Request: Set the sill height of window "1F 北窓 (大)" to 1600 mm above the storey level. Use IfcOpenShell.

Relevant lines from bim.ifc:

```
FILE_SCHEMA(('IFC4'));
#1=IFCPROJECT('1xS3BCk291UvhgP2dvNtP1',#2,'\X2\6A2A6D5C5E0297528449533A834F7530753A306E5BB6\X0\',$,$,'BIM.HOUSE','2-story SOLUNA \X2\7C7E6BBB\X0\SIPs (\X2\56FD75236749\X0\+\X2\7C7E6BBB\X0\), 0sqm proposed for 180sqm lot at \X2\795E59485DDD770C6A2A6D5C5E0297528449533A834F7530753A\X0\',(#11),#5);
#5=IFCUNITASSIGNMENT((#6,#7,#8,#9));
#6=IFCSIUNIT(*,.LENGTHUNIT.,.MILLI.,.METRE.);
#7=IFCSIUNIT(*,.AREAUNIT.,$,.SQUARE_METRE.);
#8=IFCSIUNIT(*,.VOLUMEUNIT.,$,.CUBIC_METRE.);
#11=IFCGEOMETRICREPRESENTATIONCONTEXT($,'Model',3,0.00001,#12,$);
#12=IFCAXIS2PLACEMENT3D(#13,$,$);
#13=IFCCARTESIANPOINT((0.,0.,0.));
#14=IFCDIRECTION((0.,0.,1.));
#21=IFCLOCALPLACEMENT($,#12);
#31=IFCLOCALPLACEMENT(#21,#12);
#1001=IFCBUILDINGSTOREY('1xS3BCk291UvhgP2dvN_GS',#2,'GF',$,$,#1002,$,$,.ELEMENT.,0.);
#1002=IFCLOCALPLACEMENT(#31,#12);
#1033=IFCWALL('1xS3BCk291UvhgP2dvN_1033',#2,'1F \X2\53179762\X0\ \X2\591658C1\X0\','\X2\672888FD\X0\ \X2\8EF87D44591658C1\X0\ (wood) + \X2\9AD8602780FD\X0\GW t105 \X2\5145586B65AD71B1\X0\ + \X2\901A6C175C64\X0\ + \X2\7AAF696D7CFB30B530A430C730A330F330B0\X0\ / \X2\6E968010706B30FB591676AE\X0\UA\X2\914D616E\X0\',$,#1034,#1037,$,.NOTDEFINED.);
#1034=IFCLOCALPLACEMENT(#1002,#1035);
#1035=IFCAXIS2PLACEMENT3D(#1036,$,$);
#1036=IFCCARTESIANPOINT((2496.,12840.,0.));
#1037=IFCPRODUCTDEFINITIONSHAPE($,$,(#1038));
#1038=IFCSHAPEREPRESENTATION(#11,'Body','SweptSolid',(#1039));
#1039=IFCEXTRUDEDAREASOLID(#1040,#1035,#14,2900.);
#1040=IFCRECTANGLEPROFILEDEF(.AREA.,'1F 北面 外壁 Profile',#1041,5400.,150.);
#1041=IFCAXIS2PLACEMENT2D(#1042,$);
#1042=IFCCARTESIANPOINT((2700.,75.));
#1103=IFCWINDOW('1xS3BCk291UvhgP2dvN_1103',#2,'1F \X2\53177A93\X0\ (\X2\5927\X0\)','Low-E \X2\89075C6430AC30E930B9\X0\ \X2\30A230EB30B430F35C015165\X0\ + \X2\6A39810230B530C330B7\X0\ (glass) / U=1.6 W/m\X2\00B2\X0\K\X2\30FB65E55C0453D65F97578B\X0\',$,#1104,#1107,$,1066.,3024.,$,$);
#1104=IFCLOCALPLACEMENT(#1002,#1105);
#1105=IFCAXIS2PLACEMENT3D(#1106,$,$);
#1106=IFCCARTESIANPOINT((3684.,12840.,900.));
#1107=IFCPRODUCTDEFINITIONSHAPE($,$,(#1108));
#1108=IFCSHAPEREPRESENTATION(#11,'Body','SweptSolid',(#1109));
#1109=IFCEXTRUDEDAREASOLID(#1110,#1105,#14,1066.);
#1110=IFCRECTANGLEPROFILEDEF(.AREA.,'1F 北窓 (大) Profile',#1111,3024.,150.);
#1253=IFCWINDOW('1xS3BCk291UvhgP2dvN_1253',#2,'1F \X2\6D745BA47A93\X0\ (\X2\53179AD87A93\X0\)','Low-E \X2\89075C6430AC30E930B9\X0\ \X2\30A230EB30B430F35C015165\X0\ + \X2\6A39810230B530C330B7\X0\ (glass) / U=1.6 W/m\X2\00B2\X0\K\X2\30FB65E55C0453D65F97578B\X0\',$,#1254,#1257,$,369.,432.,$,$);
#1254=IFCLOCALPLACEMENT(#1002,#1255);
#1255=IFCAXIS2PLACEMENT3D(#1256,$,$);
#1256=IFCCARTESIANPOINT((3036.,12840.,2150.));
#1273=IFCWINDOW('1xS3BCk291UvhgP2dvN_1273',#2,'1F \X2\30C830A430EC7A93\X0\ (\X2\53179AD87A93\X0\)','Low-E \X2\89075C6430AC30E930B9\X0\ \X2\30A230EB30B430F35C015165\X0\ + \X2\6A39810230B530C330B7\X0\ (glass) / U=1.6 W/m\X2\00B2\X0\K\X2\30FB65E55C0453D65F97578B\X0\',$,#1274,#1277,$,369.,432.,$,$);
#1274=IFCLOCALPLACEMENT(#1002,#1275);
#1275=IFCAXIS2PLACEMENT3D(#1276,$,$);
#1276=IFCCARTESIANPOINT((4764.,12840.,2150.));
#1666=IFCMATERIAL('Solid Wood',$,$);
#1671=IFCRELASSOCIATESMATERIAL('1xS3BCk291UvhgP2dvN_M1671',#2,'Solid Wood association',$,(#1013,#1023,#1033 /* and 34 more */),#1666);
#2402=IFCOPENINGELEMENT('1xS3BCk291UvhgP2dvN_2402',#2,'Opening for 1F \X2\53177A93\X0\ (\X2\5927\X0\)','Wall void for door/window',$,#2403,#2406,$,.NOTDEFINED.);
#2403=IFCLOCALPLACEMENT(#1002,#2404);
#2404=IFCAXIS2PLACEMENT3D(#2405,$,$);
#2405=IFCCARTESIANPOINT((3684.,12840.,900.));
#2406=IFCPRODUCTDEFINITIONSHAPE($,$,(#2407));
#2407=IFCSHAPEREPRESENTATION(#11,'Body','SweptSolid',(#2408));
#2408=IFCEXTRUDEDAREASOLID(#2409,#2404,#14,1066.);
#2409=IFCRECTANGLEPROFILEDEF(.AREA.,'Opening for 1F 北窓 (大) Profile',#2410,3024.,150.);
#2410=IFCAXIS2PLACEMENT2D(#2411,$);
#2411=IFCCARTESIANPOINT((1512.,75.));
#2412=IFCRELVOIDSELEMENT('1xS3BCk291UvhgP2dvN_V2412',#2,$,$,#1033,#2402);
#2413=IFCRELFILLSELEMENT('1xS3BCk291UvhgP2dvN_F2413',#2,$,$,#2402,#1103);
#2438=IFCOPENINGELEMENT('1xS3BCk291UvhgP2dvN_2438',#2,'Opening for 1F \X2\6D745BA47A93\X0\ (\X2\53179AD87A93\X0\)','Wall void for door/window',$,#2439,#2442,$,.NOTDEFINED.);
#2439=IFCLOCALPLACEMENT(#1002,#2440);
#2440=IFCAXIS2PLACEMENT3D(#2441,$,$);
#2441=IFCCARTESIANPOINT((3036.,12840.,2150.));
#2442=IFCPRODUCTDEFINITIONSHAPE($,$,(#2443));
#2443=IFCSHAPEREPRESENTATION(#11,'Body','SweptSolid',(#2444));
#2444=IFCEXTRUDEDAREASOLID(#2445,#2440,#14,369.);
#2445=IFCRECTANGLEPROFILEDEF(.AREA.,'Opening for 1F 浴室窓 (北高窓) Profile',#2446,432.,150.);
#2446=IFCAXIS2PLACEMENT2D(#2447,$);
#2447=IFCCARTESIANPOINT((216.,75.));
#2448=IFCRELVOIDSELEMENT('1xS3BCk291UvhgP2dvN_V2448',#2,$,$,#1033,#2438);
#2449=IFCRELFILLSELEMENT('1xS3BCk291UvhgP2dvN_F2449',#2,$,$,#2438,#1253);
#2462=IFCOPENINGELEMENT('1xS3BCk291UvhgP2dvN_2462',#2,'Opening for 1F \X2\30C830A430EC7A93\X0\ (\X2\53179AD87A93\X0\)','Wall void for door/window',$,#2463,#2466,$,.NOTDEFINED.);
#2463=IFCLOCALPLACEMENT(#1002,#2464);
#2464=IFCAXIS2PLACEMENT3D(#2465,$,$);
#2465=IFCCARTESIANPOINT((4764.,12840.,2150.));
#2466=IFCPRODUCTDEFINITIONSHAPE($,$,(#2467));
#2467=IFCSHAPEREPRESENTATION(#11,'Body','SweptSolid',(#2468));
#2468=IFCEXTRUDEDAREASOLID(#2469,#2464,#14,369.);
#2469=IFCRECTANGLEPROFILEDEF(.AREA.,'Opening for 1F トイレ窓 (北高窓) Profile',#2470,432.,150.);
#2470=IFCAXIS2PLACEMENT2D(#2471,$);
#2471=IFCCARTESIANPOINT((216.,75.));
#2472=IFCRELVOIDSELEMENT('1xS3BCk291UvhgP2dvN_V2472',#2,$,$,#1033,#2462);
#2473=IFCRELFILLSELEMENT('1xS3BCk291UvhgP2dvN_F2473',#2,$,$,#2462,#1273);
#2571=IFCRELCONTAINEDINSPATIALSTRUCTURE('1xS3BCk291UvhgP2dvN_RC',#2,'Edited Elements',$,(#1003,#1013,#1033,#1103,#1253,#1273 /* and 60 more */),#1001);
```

```python
import numpy as np
import ifcopenshell
import ifcopenshell.api.geometry
import ifcopenshell.geom
import ifcopenshell.util.element
import ifcopenshell.util.placement
import ifcopenshell.util.shape
import ifcopenshell.util.unit

model = ifcopenshell.open("bim.ifc")
unit_scale = ifcopenshell.util.unit.calculate_unit_scale(model)

window = model.by_guid("1xS3BCk291UvhgP2dvN_1103")
opening = window.FillsVoids[0].RelatingOpeningElement
storey = ifcopenshell.util.element.get_container(window, ifc_class="IfcBuildingStorey")
level = ifcopenshell.util.placement.get_local_placement(storey.ObjectPlacement)[2, 3]

# The opening's origin need not be at the sill, so measure its lowest point.
shape = ifcopenshell.geom.create_shape(ifcopenshell.geom.settings(), opening)
bottom = ifcopenshell.util.shape.get_shape_bottom_elevation(shape, shape.geometry) / unit_scale
dz = level + 1.6 / unit_scale - bottom

shift = np.array([0.0, 0.0, dz])
# The window is not placed relative to its opening, so move both.
for product in (opening, window):
    matrix = ifcopenshell.util.placement.get_local_placement(product.ObjectPlacement)
    matrix[:3, 3] += shift
    ifcopenshell.api.geometry.edit_object_placement(model, product=product, matrix=matrix, is_si=False)

print(f"moved by {dz * unit_scale:+.3f} m")

model.write("bim_edited.ifc")
```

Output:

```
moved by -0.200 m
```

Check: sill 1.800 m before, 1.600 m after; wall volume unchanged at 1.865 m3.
